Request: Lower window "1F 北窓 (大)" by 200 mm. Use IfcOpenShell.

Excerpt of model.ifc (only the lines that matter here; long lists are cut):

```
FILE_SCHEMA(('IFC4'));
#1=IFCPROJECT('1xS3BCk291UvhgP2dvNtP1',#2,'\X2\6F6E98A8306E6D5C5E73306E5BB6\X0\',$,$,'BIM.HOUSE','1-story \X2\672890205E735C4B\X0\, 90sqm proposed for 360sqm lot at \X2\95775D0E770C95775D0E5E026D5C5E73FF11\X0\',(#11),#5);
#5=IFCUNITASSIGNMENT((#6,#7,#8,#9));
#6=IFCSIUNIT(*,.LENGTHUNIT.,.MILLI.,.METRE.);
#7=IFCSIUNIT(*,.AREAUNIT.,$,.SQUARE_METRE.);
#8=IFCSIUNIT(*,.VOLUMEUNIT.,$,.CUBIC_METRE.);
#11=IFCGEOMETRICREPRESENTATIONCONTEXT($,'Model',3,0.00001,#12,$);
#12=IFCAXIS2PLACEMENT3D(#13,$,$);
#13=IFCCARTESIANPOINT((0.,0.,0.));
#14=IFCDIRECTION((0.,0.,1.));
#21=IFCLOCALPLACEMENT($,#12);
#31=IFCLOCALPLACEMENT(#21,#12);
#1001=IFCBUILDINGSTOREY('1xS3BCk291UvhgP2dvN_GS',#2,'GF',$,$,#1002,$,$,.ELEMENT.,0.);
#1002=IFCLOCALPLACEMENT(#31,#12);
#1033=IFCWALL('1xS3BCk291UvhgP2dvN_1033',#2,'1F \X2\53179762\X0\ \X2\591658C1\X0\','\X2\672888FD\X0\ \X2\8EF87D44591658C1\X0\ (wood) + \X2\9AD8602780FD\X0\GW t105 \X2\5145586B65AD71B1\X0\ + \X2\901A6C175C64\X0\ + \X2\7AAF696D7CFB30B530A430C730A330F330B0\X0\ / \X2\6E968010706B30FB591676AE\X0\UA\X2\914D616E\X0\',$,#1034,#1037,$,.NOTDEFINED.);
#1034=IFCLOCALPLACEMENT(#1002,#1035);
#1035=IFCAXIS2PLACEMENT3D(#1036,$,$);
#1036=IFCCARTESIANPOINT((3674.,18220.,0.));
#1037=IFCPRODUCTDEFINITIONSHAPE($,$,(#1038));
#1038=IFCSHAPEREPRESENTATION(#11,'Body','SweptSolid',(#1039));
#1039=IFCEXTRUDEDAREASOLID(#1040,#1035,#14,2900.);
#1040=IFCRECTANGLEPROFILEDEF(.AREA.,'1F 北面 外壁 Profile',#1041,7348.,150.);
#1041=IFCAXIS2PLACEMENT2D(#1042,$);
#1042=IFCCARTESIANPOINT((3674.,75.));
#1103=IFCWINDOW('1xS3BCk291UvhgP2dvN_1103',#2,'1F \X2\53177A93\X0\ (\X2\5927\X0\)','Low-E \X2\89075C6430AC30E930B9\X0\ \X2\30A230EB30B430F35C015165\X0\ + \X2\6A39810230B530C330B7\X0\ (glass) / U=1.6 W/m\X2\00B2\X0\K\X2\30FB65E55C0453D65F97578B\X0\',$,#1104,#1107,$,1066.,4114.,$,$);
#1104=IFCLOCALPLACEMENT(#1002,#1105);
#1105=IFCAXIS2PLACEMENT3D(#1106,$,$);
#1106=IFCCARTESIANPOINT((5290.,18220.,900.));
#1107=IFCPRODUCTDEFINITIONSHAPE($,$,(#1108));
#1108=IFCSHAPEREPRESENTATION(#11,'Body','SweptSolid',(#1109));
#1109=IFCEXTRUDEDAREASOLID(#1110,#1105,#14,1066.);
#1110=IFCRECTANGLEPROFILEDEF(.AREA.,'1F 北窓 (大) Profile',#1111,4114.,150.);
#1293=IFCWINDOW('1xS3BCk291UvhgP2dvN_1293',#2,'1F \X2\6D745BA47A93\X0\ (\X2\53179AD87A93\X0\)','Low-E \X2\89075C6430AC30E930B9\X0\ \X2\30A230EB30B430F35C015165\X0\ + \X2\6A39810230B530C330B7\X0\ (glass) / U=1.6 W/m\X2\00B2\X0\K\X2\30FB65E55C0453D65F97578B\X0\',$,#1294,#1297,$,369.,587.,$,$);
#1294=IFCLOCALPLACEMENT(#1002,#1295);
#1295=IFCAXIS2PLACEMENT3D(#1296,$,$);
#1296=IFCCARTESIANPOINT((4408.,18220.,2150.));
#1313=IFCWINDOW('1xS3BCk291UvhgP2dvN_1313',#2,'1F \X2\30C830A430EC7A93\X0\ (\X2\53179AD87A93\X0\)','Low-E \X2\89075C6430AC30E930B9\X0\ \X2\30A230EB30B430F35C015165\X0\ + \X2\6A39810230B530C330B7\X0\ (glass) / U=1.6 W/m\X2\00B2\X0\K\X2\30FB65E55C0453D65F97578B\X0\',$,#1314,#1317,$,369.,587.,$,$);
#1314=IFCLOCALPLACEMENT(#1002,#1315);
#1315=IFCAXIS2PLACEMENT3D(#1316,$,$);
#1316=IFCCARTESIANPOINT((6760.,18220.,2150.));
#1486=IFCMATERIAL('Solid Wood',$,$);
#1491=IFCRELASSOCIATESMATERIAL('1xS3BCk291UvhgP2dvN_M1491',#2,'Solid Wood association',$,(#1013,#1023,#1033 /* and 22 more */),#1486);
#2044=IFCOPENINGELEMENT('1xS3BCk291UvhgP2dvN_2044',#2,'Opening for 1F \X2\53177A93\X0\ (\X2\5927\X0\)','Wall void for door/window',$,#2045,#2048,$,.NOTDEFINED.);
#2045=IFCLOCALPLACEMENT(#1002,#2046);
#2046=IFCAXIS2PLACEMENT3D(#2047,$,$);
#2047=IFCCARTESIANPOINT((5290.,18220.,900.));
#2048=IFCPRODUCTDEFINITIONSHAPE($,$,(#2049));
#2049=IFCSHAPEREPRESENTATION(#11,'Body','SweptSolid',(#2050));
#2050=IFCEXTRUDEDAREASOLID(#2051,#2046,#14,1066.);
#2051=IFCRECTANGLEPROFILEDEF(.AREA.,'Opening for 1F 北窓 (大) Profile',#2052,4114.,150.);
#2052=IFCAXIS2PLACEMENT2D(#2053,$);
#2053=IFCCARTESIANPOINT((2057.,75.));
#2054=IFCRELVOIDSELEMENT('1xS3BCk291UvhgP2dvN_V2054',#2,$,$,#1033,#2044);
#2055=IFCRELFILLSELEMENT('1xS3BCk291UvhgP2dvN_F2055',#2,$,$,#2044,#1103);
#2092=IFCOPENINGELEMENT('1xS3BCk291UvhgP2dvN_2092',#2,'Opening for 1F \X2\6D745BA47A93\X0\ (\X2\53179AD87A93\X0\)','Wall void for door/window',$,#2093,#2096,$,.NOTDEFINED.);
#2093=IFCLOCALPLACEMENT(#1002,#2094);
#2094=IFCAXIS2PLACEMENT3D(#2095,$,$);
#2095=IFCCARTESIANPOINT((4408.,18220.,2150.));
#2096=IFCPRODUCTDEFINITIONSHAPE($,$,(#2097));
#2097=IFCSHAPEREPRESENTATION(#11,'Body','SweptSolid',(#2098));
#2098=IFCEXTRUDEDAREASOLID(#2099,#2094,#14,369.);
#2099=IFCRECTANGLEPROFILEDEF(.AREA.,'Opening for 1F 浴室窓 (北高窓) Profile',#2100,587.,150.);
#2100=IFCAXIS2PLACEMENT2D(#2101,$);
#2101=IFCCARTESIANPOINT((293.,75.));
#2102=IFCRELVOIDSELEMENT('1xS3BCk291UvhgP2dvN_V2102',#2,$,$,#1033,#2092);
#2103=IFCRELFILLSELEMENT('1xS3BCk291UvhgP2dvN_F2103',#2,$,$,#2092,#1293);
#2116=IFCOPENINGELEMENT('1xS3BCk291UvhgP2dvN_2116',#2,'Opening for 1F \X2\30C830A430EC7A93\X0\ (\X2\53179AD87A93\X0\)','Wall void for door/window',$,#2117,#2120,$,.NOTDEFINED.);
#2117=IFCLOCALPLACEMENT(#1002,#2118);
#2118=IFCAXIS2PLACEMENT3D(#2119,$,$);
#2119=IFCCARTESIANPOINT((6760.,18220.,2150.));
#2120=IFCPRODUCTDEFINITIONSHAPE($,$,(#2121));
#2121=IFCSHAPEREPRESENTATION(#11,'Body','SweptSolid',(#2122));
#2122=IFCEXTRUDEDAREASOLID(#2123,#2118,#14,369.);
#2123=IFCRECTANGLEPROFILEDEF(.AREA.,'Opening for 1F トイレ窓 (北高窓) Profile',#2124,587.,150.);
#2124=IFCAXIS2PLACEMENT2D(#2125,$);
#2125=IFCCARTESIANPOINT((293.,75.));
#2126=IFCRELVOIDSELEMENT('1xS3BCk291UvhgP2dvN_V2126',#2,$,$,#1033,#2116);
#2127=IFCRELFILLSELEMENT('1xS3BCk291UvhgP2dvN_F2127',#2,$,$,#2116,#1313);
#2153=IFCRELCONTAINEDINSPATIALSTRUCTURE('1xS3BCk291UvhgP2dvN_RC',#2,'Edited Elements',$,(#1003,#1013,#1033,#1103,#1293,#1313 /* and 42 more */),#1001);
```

```python
import numpy as np
import ifcopenshell
import ifcopenshell.api.geometry
import ifcopenshell.util.placement
import ifcopenshell.util.unit

model = ifcopenshell.open("model.ifc")
unit_scale = ifcopenshell.util.unit.calculate_unit_scale(model)

window = model.by_guid("1xS3BCk291UvhgP2dvN_1103")
opening = window.FillsVoids[0].RelatingOpeningElement
dz = -200.0

shift = np.array([0.0, 0.0, dz])
# The window is not placed relative to its opening, so move both.
for product in (opening, window):
    matrix = ifcopenshell.util.placement.get_local_placement(product.ObjectPlacement)
    matrix[:3, 3] += shift
    ifcopenshell.api.geometry.edit_object_placement(model, product=product, matrix=matrix, is_si=False)

print(f"moved by {dz * unit_scale:+.3f} m")

model.write("model_rev.ifc")
```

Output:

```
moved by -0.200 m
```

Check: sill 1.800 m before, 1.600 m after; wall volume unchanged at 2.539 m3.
